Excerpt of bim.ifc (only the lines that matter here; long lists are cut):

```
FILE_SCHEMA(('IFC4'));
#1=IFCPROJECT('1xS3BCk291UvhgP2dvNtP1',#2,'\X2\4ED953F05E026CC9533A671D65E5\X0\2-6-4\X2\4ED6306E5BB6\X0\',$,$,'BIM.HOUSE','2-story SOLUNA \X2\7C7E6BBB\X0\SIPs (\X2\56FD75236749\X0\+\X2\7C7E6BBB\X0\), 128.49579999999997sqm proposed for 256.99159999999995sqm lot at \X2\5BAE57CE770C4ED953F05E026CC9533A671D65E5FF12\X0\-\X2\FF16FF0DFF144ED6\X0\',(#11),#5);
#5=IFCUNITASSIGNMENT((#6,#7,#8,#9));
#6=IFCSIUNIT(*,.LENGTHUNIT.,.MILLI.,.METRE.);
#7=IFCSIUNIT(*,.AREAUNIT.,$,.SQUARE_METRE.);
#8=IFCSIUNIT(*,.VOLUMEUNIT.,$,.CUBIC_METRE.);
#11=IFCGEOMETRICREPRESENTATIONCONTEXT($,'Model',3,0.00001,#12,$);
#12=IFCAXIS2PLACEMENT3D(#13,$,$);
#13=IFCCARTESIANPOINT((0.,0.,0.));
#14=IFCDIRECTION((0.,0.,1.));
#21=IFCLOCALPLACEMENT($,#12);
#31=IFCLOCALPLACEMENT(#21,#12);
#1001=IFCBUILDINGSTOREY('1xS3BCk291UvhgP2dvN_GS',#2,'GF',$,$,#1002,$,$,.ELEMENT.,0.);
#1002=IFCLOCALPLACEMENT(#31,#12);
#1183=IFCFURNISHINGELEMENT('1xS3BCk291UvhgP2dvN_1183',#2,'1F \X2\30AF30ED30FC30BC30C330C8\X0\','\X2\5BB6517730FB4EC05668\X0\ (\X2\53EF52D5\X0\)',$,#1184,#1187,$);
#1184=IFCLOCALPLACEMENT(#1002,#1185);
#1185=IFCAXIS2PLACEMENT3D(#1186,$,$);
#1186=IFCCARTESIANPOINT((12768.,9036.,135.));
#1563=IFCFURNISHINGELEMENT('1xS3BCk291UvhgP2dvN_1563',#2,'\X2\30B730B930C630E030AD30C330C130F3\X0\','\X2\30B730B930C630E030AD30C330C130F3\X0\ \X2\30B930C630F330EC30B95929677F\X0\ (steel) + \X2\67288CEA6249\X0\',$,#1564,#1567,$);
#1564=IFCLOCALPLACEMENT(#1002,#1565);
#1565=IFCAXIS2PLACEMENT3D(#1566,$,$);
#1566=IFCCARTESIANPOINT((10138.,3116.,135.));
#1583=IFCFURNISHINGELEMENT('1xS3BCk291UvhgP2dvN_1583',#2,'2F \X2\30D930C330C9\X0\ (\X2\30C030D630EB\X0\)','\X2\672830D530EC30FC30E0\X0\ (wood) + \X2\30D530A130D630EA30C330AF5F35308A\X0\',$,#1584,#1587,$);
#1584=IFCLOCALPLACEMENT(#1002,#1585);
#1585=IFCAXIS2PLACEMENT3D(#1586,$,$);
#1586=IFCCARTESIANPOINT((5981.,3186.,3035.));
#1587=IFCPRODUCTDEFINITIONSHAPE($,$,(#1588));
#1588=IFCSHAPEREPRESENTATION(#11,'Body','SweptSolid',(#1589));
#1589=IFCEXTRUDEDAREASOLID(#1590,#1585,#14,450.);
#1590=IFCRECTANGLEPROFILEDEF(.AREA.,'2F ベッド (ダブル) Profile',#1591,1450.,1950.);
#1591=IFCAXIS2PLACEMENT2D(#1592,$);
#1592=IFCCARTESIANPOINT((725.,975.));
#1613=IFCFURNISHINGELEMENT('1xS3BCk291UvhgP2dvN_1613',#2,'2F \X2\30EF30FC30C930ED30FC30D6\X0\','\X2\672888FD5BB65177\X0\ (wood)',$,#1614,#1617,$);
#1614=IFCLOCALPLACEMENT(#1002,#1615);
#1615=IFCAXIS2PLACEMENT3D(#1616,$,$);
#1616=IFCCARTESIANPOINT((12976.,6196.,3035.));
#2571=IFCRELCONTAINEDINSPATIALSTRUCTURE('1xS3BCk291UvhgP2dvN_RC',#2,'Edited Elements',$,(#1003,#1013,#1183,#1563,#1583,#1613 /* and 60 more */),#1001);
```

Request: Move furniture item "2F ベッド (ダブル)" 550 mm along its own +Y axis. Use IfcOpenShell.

```python
import ifcopenshell
import ifcopenshell.api.geometry
import ifcopenshell.util.placement

model = ifcopenshell.open("bim.ifc")

item = model.by_guid("1xS3BCk291UvhgP2dvN_1583")
matrix = ifcopenshell.util.placement.get_local_placement(item.ObjectPlacement)
matrix[:3, 3] += matrix[:3, 1] * 550.0
ifcopenshell.api.geometry.edit_object_placement(model, product=item, matrix=matrix, is_si=False)

print(ifcopenshell.util.placement.get_local_placement(item.ObjectPlacement).round(3) + 0.0)

model.write("bim-out.ifc")
```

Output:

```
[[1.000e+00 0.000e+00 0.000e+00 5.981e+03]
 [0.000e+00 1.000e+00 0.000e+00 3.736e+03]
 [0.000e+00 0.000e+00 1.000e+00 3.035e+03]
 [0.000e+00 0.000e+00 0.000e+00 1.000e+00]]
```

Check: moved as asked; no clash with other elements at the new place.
